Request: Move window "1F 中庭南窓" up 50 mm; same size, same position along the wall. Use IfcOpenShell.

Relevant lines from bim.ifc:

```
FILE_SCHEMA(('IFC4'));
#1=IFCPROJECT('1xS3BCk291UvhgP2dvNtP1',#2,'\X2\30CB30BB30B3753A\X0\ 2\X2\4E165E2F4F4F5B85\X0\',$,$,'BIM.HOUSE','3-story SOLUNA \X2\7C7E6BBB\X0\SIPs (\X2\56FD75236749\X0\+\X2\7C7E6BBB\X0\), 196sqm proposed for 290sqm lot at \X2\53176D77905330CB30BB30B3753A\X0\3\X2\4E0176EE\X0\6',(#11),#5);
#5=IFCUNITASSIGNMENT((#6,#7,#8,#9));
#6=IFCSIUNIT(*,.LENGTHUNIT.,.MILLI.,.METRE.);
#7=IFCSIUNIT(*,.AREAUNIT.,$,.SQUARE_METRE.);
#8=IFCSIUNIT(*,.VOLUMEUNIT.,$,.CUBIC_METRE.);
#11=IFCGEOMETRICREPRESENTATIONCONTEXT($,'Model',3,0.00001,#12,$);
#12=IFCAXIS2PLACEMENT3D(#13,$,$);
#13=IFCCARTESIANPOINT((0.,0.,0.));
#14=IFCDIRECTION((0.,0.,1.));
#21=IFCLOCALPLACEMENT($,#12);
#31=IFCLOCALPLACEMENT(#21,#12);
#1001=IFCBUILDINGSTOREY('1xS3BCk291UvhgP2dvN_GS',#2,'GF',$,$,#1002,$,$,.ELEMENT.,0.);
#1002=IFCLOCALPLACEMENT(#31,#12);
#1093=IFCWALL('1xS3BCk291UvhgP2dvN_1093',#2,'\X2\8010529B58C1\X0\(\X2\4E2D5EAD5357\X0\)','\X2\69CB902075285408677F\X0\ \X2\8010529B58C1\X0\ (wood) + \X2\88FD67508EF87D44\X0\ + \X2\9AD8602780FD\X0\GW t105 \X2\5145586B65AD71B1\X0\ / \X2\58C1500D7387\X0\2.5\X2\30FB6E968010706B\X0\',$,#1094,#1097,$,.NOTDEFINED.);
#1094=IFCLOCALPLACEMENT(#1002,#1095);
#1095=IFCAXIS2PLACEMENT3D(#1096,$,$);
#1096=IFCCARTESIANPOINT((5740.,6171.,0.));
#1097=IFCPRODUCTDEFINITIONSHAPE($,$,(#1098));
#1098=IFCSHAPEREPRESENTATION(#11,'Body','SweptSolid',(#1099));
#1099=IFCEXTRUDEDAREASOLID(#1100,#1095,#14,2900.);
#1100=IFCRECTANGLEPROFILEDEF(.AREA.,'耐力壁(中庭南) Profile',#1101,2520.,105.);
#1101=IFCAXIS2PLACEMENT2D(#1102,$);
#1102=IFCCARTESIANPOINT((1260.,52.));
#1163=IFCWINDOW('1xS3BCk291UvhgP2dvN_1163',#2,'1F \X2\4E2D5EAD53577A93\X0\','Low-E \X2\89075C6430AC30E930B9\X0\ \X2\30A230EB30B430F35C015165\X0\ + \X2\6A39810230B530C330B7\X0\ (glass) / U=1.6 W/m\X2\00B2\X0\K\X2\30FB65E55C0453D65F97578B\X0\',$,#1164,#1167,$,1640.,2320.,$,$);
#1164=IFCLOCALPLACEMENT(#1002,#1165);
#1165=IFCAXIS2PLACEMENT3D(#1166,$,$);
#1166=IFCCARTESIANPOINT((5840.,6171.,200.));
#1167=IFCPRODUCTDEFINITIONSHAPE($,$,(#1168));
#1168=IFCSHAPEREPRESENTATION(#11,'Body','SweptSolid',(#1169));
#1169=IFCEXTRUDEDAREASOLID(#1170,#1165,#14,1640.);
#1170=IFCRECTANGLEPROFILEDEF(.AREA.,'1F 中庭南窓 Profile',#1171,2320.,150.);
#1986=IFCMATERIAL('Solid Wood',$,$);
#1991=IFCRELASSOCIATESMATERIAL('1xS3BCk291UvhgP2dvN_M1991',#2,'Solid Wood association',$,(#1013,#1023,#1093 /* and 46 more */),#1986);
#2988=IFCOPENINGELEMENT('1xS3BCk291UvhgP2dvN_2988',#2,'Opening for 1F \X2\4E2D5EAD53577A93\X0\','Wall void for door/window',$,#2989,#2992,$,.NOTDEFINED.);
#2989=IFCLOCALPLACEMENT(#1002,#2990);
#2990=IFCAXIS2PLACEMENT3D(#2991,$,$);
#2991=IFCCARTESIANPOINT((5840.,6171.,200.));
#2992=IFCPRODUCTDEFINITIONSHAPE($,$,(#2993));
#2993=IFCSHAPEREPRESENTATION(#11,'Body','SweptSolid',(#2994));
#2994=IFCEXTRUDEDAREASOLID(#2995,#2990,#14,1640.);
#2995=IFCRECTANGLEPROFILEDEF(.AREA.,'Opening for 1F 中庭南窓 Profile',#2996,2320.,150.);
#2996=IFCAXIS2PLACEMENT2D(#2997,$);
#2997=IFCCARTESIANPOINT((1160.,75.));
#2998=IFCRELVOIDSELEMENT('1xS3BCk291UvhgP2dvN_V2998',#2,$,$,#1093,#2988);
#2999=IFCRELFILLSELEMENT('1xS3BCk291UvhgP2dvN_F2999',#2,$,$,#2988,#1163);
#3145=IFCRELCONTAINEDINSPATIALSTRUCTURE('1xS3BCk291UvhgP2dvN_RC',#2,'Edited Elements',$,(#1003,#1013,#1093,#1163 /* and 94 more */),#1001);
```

```python
import numpy as np
import ifcopenshell
import ifcopenshell.api.geometry
import ifcopenshell.util.placement
import ifcopenshell.util.unit

model = ifcopenshell.open("bim.ifc")
unit_scale = ifcopenshell.util.unit.calculate_unit_scale(model)

window = model.by_guid("1xS3BCk291UvhgP2dvN_1163")
opening = window.FillsVoids[0].RelatingOpeningElement
dz = 50.0

shift = np.array([0.0, 0.0, dz])
# The window is not placed relative to its opening, so move both.
for product in (opening, window):
    matrix = ifcopenshell.util.placement.get_local_placement(product.ObjectPlacement)
    matrix[:3, 3] += shift
    ifcopenshell.api.geometry.edit_object_placement(model, product=product, matrix=matrix, is_si=False)

print(f"moved by {dz * unit_scale:+.3f} m")

model.write("bim-out.ifc")
```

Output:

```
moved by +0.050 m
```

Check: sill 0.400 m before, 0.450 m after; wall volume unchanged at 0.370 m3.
